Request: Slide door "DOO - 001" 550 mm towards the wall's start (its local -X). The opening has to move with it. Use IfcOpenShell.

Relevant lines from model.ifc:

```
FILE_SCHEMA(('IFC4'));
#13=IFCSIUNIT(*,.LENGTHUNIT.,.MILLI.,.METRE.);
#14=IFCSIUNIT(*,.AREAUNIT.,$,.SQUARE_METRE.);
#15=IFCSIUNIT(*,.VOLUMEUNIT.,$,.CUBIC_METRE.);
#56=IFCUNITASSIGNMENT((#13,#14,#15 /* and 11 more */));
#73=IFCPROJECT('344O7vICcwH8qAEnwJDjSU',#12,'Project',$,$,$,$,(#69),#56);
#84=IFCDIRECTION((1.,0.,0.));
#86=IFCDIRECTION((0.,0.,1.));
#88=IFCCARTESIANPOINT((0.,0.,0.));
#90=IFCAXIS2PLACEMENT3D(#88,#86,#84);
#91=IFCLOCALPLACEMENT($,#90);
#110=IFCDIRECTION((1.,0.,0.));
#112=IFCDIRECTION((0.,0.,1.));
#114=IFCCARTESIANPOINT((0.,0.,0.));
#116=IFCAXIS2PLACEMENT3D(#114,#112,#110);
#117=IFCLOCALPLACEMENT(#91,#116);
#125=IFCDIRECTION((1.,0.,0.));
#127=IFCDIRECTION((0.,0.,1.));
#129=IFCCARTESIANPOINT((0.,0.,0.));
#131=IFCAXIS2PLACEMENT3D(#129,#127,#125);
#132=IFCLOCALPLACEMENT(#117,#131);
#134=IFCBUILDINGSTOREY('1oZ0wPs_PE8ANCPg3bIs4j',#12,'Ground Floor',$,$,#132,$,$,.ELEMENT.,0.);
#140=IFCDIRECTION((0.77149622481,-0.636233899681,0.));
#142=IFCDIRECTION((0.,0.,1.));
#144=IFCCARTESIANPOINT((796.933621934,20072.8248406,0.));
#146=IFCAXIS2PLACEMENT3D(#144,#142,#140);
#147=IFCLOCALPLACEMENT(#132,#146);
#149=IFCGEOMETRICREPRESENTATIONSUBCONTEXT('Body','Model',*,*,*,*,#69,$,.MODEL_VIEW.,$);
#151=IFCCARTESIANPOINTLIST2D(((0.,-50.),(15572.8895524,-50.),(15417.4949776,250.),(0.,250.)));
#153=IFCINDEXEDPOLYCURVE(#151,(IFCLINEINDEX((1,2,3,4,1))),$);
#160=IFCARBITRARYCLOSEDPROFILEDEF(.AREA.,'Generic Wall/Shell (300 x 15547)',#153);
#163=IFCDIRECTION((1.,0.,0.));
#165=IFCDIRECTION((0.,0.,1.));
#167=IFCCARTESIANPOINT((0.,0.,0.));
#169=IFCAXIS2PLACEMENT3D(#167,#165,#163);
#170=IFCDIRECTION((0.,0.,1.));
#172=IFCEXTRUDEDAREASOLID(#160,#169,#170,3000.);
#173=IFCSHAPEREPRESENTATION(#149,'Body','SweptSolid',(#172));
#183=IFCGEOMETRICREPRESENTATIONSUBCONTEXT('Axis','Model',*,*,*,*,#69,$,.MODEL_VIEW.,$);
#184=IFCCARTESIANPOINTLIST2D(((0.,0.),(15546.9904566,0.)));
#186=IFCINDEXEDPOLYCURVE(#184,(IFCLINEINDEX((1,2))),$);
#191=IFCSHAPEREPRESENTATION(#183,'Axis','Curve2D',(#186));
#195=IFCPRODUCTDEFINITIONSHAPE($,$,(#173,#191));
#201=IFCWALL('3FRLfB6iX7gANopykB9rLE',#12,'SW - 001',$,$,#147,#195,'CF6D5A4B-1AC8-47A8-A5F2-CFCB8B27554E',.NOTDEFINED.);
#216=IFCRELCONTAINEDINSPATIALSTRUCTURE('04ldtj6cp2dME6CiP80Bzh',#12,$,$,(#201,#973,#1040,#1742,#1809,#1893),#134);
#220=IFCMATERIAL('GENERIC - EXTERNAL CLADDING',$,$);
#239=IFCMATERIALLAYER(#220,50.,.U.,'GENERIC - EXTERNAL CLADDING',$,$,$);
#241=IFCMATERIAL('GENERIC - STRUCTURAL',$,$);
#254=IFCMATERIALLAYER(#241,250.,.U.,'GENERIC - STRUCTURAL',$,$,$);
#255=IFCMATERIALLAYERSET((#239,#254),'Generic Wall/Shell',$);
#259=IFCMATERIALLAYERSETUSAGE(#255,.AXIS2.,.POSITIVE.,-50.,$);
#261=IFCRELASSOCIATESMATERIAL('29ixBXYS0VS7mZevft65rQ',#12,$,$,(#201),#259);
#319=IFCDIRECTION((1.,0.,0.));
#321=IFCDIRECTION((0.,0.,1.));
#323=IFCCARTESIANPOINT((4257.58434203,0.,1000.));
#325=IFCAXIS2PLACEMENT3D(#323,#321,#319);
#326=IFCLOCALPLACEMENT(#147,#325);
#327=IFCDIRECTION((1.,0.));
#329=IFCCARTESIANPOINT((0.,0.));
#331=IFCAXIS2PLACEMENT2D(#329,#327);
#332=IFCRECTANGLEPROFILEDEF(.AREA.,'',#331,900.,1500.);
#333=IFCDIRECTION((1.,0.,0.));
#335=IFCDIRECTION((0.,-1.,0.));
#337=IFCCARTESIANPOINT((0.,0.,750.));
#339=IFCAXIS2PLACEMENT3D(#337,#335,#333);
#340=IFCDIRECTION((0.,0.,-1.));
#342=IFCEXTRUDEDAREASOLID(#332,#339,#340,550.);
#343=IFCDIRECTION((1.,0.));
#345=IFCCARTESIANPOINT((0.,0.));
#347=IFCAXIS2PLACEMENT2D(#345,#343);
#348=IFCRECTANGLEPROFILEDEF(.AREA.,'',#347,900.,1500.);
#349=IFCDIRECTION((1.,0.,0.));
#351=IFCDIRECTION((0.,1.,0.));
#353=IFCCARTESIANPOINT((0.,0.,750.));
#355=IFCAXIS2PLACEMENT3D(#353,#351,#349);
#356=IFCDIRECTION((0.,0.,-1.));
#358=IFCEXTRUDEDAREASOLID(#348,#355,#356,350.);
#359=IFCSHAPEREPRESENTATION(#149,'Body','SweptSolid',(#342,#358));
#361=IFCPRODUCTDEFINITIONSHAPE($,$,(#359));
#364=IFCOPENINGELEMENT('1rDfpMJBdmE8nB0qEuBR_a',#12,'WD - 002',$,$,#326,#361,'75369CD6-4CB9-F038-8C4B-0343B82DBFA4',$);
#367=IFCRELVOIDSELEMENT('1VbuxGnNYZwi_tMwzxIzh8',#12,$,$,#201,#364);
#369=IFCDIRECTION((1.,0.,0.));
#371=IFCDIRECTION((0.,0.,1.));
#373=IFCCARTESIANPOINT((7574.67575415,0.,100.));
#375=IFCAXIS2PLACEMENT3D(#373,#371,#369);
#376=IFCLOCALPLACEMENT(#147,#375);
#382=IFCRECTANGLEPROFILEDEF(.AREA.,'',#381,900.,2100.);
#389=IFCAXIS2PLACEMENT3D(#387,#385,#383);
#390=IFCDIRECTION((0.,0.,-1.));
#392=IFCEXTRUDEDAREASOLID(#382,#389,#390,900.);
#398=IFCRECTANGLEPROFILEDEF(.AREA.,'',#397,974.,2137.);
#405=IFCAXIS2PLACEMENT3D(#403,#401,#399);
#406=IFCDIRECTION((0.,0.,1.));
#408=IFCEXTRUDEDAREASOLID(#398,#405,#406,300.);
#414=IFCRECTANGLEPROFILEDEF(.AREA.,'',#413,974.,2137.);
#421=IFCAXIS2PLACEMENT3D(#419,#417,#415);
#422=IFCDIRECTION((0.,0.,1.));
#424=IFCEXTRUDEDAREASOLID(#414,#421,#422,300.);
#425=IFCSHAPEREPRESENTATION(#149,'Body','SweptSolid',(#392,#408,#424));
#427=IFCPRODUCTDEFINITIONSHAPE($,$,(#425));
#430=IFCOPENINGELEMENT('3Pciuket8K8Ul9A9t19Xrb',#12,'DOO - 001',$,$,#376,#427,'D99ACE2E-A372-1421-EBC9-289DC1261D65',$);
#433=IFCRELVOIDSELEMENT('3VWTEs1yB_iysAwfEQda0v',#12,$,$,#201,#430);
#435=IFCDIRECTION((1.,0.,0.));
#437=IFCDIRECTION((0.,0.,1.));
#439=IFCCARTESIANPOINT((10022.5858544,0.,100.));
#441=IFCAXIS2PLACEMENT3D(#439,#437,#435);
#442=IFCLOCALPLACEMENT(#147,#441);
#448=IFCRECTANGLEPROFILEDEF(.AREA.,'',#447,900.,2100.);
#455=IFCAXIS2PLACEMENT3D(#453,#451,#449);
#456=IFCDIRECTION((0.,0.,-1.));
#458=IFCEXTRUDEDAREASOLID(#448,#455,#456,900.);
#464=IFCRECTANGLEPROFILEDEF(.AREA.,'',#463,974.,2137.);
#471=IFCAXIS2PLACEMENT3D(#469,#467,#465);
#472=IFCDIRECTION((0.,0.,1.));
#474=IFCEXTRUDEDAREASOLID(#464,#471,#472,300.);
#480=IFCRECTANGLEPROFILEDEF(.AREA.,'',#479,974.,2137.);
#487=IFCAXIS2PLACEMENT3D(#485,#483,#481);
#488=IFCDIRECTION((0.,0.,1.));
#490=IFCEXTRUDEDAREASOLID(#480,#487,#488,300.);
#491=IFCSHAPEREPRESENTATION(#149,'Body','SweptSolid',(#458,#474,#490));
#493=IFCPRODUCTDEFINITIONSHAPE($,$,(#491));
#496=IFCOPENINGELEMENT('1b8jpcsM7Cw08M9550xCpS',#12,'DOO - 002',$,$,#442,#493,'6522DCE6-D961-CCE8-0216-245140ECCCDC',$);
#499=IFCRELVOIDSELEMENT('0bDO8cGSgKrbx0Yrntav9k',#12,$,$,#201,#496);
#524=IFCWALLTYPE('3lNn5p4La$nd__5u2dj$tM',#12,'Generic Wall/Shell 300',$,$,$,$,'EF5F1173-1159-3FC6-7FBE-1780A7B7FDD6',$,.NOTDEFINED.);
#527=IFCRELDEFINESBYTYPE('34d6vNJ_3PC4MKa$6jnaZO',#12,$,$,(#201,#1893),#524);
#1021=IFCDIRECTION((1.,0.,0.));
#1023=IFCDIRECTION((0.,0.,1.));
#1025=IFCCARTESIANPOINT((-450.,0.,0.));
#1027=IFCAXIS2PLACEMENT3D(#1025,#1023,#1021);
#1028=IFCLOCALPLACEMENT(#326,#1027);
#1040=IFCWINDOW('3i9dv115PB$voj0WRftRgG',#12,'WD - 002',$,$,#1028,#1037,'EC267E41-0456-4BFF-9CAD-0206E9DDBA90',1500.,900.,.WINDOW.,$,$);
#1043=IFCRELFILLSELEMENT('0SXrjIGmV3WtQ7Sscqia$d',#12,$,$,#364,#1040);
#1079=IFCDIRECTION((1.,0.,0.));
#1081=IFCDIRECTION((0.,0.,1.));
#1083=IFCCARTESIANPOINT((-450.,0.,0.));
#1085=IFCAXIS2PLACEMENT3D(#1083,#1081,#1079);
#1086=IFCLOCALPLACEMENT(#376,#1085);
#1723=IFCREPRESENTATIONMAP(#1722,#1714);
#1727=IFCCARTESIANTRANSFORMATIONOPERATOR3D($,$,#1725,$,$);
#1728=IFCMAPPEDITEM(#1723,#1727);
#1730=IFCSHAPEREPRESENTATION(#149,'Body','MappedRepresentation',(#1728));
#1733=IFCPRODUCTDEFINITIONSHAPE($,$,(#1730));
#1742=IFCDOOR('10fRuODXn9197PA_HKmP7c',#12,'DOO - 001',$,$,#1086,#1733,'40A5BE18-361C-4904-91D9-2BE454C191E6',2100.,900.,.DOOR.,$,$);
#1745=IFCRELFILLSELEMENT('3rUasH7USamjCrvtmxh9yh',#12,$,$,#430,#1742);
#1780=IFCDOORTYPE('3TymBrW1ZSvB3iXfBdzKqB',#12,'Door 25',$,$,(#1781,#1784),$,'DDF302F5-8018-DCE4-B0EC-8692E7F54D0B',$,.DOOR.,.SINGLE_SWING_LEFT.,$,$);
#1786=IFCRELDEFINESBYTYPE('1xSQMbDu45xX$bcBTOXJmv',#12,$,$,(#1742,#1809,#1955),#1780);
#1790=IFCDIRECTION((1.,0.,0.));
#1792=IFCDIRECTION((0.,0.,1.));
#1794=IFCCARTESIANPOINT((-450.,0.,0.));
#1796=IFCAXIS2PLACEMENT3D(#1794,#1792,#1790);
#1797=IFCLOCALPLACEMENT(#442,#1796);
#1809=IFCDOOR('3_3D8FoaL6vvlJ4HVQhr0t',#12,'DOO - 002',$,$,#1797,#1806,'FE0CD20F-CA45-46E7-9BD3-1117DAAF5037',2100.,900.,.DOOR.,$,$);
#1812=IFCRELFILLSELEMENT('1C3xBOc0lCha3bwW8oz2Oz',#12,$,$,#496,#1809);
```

```python
import ifcopenshell
import ifcopenshell.api.geometry
import ifcopenshell.util.placement
import ifcopenshell.util.unit

model = ifcopenshell.open("model.ifc")
unit_scale = ifcopenshell.util.unit.calculate_unit_scale(model)

door = model.by_guid("10fRuODXn9197PA_HKmP7c")
opening = door.FillsVoids[0].RelatingOpeningElement
wall = opening.VoidsElements[0].RelatingBuildingElement

wall_matrix = ifcopenshell.util.placement.get_local_placement(wall.ObjectPlacement)
shift = wall_matrix[:3, 0] * -0.55 / unit_scale
before = ifcopenshell.util.placement.get_local_placement(door.ObjectPlacement)[:3, 3].copy()

# The door is placed relative to its opening, so it follows when the opening moves.
matrix = ifcopenshell.util.placement.get_local_placement(opening.ObjectPlacement)
matrix[:3, 3] += shift
ifcopenshell.api.geometry.edit_object_placement(
    model, product=opening, matrix=matrix, is_si=False, should_transform_children=True
)

after = ifcopenshell.util.placement.get_local_placement(door.ObjectPlacement)[:3, 3]
print("door moved by", (after - before).round(3) + 0.0)

model.write("model_edited.ifc")
```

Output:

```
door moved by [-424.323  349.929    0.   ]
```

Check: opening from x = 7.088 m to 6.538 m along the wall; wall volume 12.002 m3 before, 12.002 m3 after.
